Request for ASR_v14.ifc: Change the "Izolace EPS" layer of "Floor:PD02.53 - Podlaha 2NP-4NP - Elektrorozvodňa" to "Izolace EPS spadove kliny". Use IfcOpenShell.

First a look at what the model holds.

```python
import ifcopenshell
import ifcopenshell.util.element

model = ifcopenshell.open("ASR_v14.ifc")
print(model.schema)
for layer_set in model.by_type("IfcMaterialLayerSet"):
    if layer_set.LayerSetName == "Floor:PD02.53 - Podlaha 2NP-4NP - Elektrorozvodňa":
        for layer in layer_set.MaterialLayers:
            print(layer.id(), layer.Material and layer.Material.Name, layer.LayerThickness, sep=" | ")
        print(len(ifcopenshell.util.element.get_elements_by_material(model, layer_set)), "elements and types use it")
print(sorted(m.Name for m in model.by_type("IfcMaterial") if m.Name)[:60])
```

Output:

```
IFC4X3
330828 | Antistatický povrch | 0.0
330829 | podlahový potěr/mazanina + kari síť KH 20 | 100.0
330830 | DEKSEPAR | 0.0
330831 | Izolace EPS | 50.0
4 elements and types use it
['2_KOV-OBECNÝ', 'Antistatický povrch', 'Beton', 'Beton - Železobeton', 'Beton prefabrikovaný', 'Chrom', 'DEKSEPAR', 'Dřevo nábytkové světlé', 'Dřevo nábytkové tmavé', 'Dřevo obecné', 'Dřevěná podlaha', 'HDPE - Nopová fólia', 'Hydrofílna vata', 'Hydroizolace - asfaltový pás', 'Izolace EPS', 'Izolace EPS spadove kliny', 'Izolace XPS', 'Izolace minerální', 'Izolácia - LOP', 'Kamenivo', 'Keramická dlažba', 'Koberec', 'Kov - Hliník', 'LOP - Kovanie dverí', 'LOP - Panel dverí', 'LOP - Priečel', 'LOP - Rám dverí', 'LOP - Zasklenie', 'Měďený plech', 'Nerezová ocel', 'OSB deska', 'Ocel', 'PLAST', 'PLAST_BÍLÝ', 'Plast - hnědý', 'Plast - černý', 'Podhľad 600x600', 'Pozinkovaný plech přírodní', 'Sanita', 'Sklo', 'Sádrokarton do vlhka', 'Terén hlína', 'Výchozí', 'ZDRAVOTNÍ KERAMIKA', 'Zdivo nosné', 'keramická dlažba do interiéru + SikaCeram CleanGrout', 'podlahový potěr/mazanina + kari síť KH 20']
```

```python
import ifcopenshell
import ifcopenshell.api.material

model = ifcopenshell.open("ASR_v14.ifc")

layer_set = next(s for s in model.by_type("IfcMaterialLayerSet") if s.LayerSetName == "Floor:PD02.53 - Podlaha 2NP-4NP - Elektrorozvodňa")
layer = next(l for l in layer_set.MaterialLayers if l.Material and l.Material.Name == "Izolace EPS")
material = next(m for m in model.by_type("IfcMaterial") if m.Name == "Izolace EPS spadove kliny")

# Point this one layer at the other material; renaming the old one would change it everywhere.
ifcopenshell.api.material.edit_layer(model, layer=layer, attributes={"Name": material.Name}, material=material)

print([l.Material.Name if l.Material else None for l in layer_set.MaterialLayers])

model.write("ASR_v14_edited.ifc")
```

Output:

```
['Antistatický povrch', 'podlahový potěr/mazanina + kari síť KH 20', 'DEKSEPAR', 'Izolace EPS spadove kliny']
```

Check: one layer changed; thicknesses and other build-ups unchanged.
